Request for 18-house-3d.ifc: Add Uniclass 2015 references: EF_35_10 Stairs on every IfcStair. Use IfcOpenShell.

First a look at what the model holds.

```python
import ifcopenshell

model = ifcopenshell.open("18-house-3d.ifc")
print(model.schema)
print("classifications:", [c.Name for c in model.by_type("IfcClassification")])
for ifc_class in ("IfcDoor", "IfcRoof", "IfcStair", "IfcWall", "IfcWindow"):
    print(ifc_class, len(model.by_type(ifc_class)))
```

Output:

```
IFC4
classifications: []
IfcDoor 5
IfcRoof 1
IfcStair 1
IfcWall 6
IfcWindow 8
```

```python
import ifcopenshell
import ifcopenshell.api.classification

model = ifcopenshell.open("18-house-3d.ifc")

system = ifcopenshell.api.classification.add_classification(model, classification="Uniclass 2015")

codes = {
    "IfcStair": ("EF_35_10", "Stairs"),
}
for ifc_class, (code, name) in codes.items():
    products = model.by_type(ifc_class)
    ifcopenshell.api.classification.add_reference(
        model, products=products, classification=system, identification=code, name=name
    )
    print(code, len(products))

model.write("18-house-3d_rev.ifc")
```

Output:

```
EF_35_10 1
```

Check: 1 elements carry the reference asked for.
